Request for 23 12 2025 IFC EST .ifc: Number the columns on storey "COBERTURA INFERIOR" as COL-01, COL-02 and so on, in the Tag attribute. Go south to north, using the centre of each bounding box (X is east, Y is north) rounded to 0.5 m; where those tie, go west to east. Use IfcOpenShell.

First a look at what the model holds.

```python
import ifcopenshell
import ifcopenshell.util.element
import ifcopenshell.util.placement

model = ifcopenshell.open("23 12 2025 IFC EST .ifc")
print(model.schema)
storey = next(s for s in model.by_type("IfcBuildingStorey") if s.Name == "COBERTURA INFERIOR")
columns = [e for e in ifcopenshell.util.element.get_decomposition(storey) if e.is_a("IfcColumn")]
for e in sorted(columns, key=lambda e: e.id()):
    origin = ifcopenshell.util.placement.get_local_placement(e.ObjectPlacement)[:3, 3]
    print(e.id(), e.Tag, e.Name, origin.round(2) + 0.0, sep=" | ")
```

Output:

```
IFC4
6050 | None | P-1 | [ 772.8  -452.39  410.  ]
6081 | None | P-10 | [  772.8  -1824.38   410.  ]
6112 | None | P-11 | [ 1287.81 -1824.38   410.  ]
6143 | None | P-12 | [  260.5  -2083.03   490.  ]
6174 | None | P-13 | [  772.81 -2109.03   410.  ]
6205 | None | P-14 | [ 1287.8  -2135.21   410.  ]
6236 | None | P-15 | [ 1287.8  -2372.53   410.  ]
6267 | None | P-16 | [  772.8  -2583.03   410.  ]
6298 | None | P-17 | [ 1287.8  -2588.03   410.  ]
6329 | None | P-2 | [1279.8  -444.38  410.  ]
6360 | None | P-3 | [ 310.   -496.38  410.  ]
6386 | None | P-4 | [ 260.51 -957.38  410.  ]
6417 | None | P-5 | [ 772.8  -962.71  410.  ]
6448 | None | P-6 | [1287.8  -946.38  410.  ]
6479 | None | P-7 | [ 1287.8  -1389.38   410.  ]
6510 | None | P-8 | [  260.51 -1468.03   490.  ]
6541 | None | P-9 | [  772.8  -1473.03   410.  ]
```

```python
import ifcopenshell
import ifcopenshell.geom
import ifcopenshell.util.element
import ifcopenshell.util.shape

model = ifcopenshell.open("23 12 2025 IFC EST .ifc")
settings = ifcopenshell.geom.settings()
settings.set("use-world-coords", True)


def centre(element):
    shape = ifcopenshell.geom.create_shape(settings, element)
    return ifcopenshell.util.shape.get_bbox_centroid(shape.geometry)


storey = next(s for s in model.by_type("IfcBuildingStorey") if s.Name == "COBERTURA INFERIOR")
columns = [e for e in ifcopenshell.util.element.get_decomposition(storey) if e.is_a("IfcColumn")]

# Insertion points can sit at a corner or the storey origin, so sort by the geometry (in metres).
centres = {e: centre(e) for e in columns}
columns.sort(key=lambda e: (round(centres[e][1] / 0.5), centres[e][0]))

for i, e in enumerate(columns, start=1):
    number = f"COL-{i:02d}"
    e.Tag = number
    print(e.id(), number)

model.write("23 12 2025 IFC EST _edited.ifc")
```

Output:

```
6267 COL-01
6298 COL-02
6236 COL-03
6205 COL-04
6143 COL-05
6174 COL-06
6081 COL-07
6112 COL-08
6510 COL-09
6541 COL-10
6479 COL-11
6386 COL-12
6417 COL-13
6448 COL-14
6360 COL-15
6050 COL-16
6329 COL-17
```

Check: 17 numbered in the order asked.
